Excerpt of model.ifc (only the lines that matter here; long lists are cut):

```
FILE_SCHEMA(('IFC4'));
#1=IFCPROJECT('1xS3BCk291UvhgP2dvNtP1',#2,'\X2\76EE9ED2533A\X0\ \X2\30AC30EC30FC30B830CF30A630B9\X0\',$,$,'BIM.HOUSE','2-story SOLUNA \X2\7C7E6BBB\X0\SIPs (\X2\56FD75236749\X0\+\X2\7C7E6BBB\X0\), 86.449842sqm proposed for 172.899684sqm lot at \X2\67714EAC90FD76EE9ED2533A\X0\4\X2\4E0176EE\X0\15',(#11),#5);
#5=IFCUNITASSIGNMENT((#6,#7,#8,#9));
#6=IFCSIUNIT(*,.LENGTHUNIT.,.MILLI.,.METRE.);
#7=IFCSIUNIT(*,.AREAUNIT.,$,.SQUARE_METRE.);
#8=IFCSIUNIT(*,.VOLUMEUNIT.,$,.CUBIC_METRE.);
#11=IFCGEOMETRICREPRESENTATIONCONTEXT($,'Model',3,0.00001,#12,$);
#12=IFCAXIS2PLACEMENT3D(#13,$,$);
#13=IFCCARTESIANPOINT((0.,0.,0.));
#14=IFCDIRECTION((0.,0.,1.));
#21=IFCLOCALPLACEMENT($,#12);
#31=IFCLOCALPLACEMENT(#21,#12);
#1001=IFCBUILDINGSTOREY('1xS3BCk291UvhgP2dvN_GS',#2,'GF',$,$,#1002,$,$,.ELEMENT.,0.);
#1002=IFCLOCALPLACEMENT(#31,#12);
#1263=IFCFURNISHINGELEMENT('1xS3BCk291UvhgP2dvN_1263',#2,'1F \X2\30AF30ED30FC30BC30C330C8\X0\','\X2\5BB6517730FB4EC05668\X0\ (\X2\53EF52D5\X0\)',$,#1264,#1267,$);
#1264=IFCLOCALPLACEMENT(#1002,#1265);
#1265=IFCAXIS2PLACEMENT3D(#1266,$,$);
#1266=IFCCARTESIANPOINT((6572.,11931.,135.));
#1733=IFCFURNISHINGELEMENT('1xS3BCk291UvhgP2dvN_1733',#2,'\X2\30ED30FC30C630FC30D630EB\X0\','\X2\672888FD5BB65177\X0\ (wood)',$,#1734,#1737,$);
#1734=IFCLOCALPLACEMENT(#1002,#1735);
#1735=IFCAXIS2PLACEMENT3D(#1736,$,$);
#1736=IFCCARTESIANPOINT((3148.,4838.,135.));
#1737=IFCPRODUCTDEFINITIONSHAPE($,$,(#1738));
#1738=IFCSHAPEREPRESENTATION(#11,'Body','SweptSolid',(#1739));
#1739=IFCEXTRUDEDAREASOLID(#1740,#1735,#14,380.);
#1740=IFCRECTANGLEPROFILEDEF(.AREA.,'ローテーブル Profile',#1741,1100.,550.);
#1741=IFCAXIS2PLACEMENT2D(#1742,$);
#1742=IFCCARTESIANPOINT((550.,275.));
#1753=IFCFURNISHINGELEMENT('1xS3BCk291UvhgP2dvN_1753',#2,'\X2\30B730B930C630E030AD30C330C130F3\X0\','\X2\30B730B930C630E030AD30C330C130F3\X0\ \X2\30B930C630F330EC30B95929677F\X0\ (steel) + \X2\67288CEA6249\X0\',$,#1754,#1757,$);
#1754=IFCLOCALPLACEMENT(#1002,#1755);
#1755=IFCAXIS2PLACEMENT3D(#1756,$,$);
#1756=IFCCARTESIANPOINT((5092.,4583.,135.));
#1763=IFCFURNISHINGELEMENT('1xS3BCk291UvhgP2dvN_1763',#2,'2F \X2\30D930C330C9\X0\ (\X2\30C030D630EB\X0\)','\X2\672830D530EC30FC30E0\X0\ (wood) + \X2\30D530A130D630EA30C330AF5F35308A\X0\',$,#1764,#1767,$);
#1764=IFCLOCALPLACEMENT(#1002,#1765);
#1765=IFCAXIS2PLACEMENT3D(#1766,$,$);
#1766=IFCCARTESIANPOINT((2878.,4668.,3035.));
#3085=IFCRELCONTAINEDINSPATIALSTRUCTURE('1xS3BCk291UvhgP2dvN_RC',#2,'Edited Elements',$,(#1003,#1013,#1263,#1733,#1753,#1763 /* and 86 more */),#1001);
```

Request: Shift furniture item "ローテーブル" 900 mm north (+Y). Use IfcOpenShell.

```python
import ifcopenshell
import ifcopenshell.api.geometry
import ifcopenshell.util.placement

model = ifcopenshell.open("model.ifc")

item = model.by_guid("1xS3BCk291UvhgP2dvN_1733")
matrix = ifcopenshell.util.placement.get_local_placement(item.ObjectPlacement)
matrix[1, 3] += 900.0
ifcopenshell.api.geometry.edit_object_placement(model, product=item, matrix=matrix, is_si=False)

print(ifcopenshell.util.placement.get_local_placement(item.ObjectPlacement).round(3) + 0.0)

model.write("model_updated.ifc")
```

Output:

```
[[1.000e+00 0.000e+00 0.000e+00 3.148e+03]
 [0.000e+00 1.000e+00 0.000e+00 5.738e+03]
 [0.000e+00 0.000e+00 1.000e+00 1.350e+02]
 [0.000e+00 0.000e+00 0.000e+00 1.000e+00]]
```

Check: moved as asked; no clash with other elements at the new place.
